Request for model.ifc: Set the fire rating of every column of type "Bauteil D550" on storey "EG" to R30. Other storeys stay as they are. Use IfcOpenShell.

First a look at what the model holds.

```python
import ifcopenshell
import ifcopenshell.util.element

model = ifcopenshell.open("model.ifc")
print(model.schema)
storey = next(s for s in model.by_type("IfcBuildingStorey") if s.Name == "EG")
columns = [e for e in ifcopenshell.util.element.get_decomposition(storey) if e.is_a("IfcColumn")]
seen = {}
for e in columns:
    element_type = ifcopenshell.util.element.get_type(e)
    key = (element_type.Name if element_type != e and element_type else None, ifcopenshell.util.element.get_pset(e, "Pset_ColumnCommon", "FireRating"))
    seen[key] = seen.get(key, 0) + 1
for (name, value), count in sorted(seen.items(), key=str):
    print(count, "x", name, "|", value)
```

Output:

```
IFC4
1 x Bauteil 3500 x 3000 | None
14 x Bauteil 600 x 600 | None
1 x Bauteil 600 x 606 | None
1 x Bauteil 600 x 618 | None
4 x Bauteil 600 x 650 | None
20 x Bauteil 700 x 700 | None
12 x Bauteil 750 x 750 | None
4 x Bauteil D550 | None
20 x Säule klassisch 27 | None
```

```python
import ifcopenshell
import ifcopenshell.api.pset
import ifcopenshell.util.element

model = ifcopenshell.open("model.ifc")

storey = next(s for s in model.by_type("IfcBuildingStorey") if s.Name == "EG")
columns = [e for e in ifcopenshell.util.element.get_decomposition(storey) if e.is_a("IfcColumn")]

count = 0
for e in columns:
    element_type = ifcopenshell.util.element.get_type(e)
    if element_type in (None, e) or element_type.Name != "Bauteil D550":
        continue
    # add_pset returns the element's existing set when there is one.
    pset = ifcopenshell.api.pset.add_pset(model, product=e, name="Pset_ColumnCommon")
    ifcopenshell.api.pset.edit_pset(model, pset=pset, properties={"FireRating": "R30"})
    count += 1

print(count, "columns updated")

model.write("model_updated.ifc")
```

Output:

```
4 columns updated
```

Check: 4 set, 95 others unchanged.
